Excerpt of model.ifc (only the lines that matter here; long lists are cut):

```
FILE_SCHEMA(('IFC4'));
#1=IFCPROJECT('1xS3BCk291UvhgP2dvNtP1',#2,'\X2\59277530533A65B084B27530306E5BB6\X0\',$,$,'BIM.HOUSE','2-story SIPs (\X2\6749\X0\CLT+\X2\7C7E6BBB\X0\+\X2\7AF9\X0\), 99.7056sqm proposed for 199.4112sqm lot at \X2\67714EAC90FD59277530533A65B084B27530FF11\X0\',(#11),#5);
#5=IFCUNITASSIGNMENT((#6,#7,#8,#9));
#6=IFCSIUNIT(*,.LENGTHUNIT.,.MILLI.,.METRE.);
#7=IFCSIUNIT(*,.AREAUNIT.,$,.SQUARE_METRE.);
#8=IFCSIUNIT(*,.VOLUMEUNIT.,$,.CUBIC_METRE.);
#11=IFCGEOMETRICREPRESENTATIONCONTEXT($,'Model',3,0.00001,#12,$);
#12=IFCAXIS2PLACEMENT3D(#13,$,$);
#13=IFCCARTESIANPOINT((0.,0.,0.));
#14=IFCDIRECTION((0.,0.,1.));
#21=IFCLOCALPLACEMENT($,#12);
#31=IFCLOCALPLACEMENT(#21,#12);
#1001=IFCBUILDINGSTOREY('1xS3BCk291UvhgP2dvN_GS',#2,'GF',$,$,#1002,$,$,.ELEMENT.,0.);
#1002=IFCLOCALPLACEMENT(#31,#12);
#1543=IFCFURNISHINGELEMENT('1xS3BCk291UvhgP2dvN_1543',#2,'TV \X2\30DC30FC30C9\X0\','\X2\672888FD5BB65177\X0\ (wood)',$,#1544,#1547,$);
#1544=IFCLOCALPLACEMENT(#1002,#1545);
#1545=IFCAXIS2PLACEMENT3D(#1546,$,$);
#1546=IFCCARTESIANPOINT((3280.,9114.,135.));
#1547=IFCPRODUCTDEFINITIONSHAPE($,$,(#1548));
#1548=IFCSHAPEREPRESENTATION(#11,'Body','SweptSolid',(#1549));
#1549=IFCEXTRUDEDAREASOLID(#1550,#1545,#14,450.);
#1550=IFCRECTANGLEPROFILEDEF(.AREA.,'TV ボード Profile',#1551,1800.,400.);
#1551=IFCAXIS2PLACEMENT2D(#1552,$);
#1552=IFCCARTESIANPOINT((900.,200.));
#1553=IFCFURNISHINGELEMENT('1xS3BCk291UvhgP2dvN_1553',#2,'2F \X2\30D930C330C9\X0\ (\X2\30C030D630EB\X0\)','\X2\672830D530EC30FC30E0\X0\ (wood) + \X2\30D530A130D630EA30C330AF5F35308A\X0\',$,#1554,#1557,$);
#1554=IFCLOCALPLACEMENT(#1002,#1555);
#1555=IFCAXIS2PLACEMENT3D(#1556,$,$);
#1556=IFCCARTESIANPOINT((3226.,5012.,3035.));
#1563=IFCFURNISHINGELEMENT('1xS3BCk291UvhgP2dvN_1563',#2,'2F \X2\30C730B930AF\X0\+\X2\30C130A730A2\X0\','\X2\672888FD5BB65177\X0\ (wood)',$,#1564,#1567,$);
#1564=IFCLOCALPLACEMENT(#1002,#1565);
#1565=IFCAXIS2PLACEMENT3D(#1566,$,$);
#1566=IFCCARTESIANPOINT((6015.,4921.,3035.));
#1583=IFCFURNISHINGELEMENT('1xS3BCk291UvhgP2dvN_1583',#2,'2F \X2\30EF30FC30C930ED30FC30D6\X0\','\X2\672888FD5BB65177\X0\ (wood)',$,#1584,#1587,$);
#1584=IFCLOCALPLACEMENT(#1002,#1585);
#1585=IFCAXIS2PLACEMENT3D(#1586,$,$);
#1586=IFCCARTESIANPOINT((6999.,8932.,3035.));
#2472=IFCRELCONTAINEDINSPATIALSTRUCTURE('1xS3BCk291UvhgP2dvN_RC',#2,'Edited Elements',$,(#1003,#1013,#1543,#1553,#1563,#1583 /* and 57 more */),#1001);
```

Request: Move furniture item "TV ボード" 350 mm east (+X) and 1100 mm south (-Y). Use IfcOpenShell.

```python
import ifcopenshell
import ifcopenshell.api.geometry
import ifcopenshell.util.placement
import ifcopenshell.util.unit

model = ifcopenshell.open("model.ifc")
unit_scale = ifcopenshell.util.unit.calculate_unit_scale(model)

item = model.by_id(1543)
matrix = ifcopenshell.util.placement.get_local_placement(item.ObjectPlacement)
matrix[0, 3] += 0.35 / unit_scale
matrix[1, 3] -= 1.1 / unit_scale
ifcopenshell.api.geometry.edit_object_placement(model, product=item, matrix=matrix, is_si=False)

print(ifcopenshell.util.placement.get_local_placement(item.ObjectPlacement).round(3) + 0.0)

model.write("model_edited.ifc")
```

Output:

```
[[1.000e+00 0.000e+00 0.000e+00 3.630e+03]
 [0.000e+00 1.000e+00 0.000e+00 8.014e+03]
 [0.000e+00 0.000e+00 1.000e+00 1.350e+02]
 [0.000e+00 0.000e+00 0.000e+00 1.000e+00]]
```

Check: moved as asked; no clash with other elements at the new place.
